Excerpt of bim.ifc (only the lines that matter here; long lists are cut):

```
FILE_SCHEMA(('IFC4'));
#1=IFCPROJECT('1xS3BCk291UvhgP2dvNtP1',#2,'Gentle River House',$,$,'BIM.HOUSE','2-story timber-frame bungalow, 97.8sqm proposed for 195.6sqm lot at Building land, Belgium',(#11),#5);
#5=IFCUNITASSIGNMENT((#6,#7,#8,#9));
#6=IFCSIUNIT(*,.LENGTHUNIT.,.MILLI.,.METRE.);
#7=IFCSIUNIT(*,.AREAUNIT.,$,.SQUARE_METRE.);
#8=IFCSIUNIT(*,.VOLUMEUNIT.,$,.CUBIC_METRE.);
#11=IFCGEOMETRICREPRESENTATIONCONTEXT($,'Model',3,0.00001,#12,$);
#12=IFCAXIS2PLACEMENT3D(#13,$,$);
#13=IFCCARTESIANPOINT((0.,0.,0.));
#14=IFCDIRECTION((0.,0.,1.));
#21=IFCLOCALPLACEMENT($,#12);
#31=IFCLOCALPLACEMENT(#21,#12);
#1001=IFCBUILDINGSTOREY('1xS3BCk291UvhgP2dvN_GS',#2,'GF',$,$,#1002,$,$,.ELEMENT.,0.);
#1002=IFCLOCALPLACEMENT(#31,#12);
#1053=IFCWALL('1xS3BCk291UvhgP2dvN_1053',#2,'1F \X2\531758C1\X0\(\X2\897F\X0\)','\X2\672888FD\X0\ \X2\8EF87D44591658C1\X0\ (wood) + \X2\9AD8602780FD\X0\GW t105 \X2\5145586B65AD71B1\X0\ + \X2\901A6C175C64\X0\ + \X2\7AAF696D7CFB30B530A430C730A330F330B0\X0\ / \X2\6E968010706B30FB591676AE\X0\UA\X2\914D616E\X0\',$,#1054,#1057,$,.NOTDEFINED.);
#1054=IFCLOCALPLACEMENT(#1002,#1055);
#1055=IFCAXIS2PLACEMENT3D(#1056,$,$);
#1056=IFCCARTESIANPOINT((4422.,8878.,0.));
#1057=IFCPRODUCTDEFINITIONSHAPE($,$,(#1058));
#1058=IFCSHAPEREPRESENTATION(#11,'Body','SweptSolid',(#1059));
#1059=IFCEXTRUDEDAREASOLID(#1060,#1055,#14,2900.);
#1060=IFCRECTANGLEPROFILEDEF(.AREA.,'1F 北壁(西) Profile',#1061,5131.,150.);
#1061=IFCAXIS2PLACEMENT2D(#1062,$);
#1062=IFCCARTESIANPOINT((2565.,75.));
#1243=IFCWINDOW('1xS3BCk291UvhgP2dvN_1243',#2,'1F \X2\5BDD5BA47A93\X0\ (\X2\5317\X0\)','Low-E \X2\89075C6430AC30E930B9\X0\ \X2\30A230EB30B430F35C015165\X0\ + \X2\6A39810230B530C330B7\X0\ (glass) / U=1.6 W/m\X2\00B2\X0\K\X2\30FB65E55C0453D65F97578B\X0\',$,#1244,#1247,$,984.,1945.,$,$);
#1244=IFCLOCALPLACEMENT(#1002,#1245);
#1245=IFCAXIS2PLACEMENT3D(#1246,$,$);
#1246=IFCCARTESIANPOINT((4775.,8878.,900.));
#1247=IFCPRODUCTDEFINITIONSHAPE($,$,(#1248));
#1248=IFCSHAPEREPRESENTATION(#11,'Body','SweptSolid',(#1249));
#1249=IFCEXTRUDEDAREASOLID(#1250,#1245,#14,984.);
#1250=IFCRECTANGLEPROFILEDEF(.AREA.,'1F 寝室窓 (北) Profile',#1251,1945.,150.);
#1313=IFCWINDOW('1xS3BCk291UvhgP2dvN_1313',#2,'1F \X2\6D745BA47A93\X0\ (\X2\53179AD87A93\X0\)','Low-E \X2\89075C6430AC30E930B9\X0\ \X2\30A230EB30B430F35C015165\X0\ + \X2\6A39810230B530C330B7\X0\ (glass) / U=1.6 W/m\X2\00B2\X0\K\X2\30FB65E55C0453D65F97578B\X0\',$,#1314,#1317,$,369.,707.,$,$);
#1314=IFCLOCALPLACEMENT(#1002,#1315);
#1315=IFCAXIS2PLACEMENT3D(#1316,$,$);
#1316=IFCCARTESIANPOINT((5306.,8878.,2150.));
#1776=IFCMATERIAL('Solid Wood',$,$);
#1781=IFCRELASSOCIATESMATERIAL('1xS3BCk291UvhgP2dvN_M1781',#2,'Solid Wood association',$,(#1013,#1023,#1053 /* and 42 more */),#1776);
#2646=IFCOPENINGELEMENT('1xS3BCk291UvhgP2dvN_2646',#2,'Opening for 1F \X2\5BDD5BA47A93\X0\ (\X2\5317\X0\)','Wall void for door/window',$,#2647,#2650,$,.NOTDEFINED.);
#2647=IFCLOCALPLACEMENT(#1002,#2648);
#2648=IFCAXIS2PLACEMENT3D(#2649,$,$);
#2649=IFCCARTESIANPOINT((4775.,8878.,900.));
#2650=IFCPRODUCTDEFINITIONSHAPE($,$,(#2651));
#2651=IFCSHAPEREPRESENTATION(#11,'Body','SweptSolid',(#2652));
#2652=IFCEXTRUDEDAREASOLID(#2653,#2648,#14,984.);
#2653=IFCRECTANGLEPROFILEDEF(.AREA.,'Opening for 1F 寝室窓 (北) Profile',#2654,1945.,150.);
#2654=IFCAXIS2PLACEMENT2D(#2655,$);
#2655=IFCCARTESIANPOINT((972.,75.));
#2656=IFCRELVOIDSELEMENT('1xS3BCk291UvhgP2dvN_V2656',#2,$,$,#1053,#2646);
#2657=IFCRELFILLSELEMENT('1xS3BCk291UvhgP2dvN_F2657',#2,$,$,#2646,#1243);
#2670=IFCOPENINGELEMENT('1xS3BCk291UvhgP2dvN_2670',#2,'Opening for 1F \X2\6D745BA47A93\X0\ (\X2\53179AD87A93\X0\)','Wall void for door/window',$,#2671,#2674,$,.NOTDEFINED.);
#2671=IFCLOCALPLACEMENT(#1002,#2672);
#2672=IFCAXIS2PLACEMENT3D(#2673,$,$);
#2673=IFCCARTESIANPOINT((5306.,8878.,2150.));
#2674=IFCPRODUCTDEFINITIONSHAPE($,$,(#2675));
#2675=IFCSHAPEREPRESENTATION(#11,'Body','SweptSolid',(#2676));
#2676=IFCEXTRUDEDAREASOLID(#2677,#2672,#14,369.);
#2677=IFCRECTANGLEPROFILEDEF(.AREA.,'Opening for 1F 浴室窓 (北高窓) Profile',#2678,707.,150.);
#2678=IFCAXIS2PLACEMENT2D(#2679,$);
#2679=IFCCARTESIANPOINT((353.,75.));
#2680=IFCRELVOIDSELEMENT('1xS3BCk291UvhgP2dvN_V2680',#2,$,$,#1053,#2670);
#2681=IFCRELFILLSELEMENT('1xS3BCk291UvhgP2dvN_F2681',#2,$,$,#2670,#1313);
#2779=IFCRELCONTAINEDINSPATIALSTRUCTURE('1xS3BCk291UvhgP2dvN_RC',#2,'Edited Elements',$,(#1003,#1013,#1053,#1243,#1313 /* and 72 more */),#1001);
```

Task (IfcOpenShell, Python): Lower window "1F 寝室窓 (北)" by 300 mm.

```python
import numpy as np
import ifcopenshell
import ifcopenshell.api.geometry
import ifcopenshell.util.placement
import ifcopenshell.util.unit

model = ifcopenshell.open("bim.ifc")
unit_scale = ifcopenshell.util.unit.calculate_unit_scale(model)

window = model.by_id(1243)
opening = window.FillsVoids[0].RelatingOpeningElement
dz = -0.3 / unit_scale

shift = np.array([0.0, 0.0, dz])
# The window is not placed relative to its opening, so move both.
for product in (opening, window):
    matrix = ifcopenshell.util.placement.get_local_placement(product.ObjectPlacement)
    matrix[:3, 3] += shift
    ifcopenshell.api.geometry.edit_object_placement(model, product=product, matrix=matrix, is_si=False)

print(f"moved by {dz * unit_scale:+.3f} m")

model.write("bim_rev.ifc")
```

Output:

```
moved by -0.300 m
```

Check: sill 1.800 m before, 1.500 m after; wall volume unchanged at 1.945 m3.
